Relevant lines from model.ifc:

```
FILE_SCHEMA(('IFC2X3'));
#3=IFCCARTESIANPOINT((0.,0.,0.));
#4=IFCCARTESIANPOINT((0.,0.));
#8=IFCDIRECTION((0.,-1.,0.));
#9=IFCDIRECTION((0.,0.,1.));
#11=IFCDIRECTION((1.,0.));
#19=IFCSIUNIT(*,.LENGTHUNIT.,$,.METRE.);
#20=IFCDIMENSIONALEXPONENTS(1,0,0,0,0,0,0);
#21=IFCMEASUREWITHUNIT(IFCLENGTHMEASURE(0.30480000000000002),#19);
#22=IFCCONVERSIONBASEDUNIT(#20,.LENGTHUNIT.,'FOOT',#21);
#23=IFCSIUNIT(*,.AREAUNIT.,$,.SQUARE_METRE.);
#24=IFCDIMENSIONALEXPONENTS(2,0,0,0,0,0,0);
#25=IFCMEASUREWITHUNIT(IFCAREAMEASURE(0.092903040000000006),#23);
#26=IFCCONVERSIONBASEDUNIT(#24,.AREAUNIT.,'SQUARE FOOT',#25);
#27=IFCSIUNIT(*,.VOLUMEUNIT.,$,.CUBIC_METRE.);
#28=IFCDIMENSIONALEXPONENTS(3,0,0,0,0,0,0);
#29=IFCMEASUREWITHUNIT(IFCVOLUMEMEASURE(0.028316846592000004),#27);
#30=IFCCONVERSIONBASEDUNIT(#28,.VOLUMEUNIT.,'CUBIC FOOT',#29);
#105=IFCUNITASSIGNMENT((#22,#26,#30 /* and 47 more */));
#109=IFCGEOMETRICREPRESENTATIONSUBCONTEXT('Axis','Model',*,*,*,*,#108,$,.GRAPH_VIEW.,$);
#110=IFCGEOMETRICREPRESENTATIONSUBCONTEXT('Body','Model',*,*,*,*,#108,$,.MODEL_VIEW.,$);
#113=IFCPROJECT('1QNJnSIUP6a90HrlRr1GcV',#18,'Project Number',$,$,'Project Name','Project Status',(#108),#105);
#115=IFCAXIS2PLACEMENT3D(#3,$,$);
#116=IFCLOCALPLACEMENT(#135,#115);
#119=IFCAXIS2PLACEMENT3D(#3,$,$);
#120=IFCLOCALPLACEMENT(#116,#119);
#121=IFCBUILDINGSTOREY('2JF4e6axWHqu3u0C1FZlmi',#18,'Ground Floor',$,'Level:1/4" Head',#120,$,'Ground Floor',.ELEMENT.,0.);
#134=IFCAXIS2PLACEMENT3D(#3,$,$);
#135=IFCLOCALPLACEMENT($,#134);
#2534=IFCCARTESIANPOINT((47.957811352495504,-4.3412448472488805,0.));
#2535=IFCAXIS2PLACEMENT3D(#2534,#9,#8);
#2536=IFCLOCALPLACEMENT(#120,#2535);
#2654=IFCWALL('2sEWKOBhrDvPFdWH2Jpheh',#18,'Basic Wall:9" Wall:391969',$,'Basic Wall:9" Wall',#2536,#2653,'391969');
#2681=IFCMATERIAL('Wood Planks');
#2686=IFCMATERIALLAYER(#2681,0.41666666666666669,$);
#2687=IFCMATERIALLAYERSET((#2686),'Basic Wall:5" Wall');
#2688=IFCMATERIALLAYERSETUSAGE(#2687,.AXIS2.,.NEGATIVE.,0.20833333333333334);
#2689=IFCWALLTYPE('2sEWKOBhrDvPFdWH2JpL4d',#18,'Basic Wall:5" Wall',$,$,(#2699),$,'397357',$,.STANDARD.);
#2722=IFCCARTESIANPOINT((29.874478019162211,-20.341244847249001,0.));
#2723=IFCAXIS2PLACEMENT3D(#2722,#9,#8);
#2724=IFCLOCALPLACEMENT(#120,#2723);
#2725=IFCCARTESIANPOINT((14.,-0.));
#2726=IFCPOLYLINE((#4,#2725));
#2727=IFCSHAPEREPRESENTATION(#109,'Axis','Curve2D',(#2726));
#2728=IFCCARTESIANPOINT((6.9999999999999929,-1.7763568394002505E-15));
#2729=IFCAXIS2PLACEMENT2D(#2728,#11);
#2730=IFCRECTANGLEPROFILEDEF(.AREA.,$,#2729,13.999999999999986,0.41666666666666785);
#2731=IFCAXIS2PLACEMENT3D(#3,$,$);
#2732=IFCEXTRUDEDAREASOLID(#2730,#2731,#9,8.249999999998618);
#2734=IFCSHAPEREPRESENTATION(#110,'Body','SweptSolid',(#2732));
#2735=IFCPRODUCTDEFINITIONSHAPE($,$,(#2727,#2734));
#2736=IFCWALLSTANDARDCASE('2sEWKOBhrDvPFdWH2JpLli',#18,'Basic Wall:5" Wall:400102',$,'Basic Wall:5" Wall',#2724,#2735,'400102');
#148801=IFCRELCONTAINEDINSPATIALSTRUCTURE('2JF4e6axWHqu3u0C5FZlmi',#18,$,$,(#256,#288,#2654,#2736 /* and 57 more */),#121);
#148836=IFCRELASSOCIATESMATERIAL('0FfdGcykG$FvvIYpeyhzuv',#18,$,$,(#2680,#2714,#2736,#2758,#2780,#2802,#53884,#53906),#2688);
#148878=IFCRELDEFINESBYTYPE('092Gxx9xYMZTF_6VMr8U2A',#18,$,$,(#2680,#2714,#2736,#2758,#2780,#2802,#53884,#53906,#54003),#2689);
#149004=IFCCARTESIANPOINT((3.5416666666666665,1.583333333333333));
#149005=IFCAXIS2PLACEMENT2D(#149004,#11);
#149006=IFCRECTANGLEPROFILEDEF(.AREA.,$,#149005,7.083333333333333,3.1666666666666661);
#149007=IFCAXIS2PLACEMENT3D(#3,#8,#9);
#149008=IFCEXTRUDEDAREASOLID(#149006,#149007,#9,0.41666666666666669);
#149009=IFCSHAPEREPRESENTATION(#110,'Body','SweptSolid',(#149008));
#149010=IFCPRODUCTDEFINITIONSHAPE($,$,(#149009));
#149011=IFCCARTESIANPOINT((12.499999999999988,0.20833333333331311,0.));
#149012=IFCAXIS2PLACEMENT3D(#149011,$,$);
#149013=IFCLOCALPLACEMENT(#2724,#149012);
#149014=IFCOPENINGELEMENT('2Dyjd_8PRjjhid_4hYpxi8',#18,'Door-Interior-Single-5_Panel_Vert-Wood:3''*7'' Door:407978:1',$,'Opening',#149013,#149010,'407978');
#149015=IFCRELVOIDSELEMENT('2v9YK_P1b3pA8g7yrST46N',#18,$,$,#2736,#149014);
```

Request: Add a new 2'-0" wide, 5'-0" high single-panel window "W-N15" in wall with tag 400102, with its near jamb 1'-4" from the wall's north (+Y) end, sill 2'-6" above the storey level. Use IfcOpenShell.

```python
import numpy as np
import ifcopenshell
import ifcopenshell.api.feature
import ifcopenshell.api.geometry
import ifcopenshell.api.root
import ifcopenshell.api.spatial
import ifcopenshell.api.type
import ifcopenshell.geom
import ifcopenshell.util.element
import ifcopenshell.util.placement
import ifcopenshell.util.representation
import ifcopenshell.util.shape
import ifcopenshell.util.unit

model = ifcopenshell.open("model.ifc")
unit_scale = ifcopenshell.util.unit.calculate_unit_scale(model)
settings = ifcopenshell.geom.settings()


def volume(element):
    """Net volume in cubic metres, openings subtracted."""
    shape = ifcopenshell.geom.create_shape(settings, element)
    return ifcopenshell.util.shape.get_volume(shape.geometry)


wall = model.by_guid("2sEWKOBhrDvPFdWH2JpLli")
storey = ifcopenshell.util.element.get_container(wall, ifc_class="IfcBuildingStorey")
context = ifcopenshell.util.representation.get_context(model, "Model", "Body", "MODEL_VIEW")
before = volume(wall)

width, height, from_end, sill = 0.6096, 1.524, 0.4064, 0.762  # metres

# The wall runs along its own X axis, and the end named is its -X end.
wall_shape = ifcopenshell.geom.create_shape(settings, wall)
x, y, z = ifcopenshell.util.shape.get_vertices(wall_shape.geometry).T
start = x.min() + from_end
face, thickness = float(y.min()), float(y.max() - y.min())
wall_matrix = ifcopenshell.util.placement.get_local_placement(wall.ObjectPlacement)
level = ifcopenshell.util.placement.get_local_placement(storey.ObjectPlacement)[2, 3]


def in_wall(x, y):
    """Placement at x, y metres in the wall's axes, at sill height."""
    matrix = wall_matrix.copy()
    matrix[:, 3] = wall_matrix @ np.array([x / unit_scale, y / unit_scale, 0.0, 1.0])
    matrix[2, 3] = level + sill / unit_scale
    return matrix


# Opening: a box that overshoots both wall faces by 50 mm.
opening = ifcopenshell.api.root.create_entity(model, ifc_class="IfcOpeningElement")
box = ifcopenshell.api.geometry.add_wall_representation(
    model, context=context, length=width, height=height, thickness=thickness + 0.1
)
ifcopenshell.api.geometry.assign_representation(model, product=opening, representation=box)
ifcopenshell.api.geometry.edit_object_placement(model, product=opening, matrix=in_wall(start, face - 0.05), is_si=False)
ifcopenshell.api.feature.add_feature(model, feature=opening, element=wall)

window = ifcopenshell.api.root.create_entity(model, ifc_class="IfcWindow", name="W-N15")
window.OverallWidth, window.OverallHeight = width / unit_scale, height / unit_scale
body = ifcopenshell.api.geometry.add_window_representation(
    model,
    context=context,
    overall_width=window.OverallWidth,
    overall_height=window.OverallHeight,
    partition_type="SINGLE_PANEL",
)
ifcopenshell.api.geometry.assign_representation(model, product=window, representation=body)
ifcopenshell.api.spatial.assign_container(model, products=[window], relating_structure=storey)
fills = ifcopenshell.api.feature.add_filling(model, opening=opening, element=window)
fills.OwnerHistory = window.OwnerHistory  # required in IFC2X3

# IFC2X3 keeps the operation on the window style.
style = ifcopenshell.api.root.create_entity(model, ifc_class="IfcWindowStyle", name="W-N15")
style.OperationType, style.ConstructionType = "SINGLE_PANEL", "NOTDEFINED"
style.ParameterTakesPrecedence = style.Sizeable = False
ifcopenshell.api.type.assign_type(model, related_objects=[window], relating_type=style)

# Centre the window in the wall's thickness.
ifcopenshell.api.geometry.edit_object_placement(model, product=window, matrix=in_wall(start, face), is_si=False)
window_shape = ifcopenshell.geom.create_shape(settings, window)
depth = ifcopenshell.util.shape.get_vertices(window_shape.geometry)[:, 1]
offset = face + thickness / 2 - (depth.min() + depth.max()) / 2
ifcopenshell.api.geometry.edit_object_placement(model, product=window, matrix=in_wall(start, offset), is_si=False)

after = volume(wall)

print(f"wall volume {before:.3f} -> {after:.3f} m3")

model.write("model-out.ifc")
```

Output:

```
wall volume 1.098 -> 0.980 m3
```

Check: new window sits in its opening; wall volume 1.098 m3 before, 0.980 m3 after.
